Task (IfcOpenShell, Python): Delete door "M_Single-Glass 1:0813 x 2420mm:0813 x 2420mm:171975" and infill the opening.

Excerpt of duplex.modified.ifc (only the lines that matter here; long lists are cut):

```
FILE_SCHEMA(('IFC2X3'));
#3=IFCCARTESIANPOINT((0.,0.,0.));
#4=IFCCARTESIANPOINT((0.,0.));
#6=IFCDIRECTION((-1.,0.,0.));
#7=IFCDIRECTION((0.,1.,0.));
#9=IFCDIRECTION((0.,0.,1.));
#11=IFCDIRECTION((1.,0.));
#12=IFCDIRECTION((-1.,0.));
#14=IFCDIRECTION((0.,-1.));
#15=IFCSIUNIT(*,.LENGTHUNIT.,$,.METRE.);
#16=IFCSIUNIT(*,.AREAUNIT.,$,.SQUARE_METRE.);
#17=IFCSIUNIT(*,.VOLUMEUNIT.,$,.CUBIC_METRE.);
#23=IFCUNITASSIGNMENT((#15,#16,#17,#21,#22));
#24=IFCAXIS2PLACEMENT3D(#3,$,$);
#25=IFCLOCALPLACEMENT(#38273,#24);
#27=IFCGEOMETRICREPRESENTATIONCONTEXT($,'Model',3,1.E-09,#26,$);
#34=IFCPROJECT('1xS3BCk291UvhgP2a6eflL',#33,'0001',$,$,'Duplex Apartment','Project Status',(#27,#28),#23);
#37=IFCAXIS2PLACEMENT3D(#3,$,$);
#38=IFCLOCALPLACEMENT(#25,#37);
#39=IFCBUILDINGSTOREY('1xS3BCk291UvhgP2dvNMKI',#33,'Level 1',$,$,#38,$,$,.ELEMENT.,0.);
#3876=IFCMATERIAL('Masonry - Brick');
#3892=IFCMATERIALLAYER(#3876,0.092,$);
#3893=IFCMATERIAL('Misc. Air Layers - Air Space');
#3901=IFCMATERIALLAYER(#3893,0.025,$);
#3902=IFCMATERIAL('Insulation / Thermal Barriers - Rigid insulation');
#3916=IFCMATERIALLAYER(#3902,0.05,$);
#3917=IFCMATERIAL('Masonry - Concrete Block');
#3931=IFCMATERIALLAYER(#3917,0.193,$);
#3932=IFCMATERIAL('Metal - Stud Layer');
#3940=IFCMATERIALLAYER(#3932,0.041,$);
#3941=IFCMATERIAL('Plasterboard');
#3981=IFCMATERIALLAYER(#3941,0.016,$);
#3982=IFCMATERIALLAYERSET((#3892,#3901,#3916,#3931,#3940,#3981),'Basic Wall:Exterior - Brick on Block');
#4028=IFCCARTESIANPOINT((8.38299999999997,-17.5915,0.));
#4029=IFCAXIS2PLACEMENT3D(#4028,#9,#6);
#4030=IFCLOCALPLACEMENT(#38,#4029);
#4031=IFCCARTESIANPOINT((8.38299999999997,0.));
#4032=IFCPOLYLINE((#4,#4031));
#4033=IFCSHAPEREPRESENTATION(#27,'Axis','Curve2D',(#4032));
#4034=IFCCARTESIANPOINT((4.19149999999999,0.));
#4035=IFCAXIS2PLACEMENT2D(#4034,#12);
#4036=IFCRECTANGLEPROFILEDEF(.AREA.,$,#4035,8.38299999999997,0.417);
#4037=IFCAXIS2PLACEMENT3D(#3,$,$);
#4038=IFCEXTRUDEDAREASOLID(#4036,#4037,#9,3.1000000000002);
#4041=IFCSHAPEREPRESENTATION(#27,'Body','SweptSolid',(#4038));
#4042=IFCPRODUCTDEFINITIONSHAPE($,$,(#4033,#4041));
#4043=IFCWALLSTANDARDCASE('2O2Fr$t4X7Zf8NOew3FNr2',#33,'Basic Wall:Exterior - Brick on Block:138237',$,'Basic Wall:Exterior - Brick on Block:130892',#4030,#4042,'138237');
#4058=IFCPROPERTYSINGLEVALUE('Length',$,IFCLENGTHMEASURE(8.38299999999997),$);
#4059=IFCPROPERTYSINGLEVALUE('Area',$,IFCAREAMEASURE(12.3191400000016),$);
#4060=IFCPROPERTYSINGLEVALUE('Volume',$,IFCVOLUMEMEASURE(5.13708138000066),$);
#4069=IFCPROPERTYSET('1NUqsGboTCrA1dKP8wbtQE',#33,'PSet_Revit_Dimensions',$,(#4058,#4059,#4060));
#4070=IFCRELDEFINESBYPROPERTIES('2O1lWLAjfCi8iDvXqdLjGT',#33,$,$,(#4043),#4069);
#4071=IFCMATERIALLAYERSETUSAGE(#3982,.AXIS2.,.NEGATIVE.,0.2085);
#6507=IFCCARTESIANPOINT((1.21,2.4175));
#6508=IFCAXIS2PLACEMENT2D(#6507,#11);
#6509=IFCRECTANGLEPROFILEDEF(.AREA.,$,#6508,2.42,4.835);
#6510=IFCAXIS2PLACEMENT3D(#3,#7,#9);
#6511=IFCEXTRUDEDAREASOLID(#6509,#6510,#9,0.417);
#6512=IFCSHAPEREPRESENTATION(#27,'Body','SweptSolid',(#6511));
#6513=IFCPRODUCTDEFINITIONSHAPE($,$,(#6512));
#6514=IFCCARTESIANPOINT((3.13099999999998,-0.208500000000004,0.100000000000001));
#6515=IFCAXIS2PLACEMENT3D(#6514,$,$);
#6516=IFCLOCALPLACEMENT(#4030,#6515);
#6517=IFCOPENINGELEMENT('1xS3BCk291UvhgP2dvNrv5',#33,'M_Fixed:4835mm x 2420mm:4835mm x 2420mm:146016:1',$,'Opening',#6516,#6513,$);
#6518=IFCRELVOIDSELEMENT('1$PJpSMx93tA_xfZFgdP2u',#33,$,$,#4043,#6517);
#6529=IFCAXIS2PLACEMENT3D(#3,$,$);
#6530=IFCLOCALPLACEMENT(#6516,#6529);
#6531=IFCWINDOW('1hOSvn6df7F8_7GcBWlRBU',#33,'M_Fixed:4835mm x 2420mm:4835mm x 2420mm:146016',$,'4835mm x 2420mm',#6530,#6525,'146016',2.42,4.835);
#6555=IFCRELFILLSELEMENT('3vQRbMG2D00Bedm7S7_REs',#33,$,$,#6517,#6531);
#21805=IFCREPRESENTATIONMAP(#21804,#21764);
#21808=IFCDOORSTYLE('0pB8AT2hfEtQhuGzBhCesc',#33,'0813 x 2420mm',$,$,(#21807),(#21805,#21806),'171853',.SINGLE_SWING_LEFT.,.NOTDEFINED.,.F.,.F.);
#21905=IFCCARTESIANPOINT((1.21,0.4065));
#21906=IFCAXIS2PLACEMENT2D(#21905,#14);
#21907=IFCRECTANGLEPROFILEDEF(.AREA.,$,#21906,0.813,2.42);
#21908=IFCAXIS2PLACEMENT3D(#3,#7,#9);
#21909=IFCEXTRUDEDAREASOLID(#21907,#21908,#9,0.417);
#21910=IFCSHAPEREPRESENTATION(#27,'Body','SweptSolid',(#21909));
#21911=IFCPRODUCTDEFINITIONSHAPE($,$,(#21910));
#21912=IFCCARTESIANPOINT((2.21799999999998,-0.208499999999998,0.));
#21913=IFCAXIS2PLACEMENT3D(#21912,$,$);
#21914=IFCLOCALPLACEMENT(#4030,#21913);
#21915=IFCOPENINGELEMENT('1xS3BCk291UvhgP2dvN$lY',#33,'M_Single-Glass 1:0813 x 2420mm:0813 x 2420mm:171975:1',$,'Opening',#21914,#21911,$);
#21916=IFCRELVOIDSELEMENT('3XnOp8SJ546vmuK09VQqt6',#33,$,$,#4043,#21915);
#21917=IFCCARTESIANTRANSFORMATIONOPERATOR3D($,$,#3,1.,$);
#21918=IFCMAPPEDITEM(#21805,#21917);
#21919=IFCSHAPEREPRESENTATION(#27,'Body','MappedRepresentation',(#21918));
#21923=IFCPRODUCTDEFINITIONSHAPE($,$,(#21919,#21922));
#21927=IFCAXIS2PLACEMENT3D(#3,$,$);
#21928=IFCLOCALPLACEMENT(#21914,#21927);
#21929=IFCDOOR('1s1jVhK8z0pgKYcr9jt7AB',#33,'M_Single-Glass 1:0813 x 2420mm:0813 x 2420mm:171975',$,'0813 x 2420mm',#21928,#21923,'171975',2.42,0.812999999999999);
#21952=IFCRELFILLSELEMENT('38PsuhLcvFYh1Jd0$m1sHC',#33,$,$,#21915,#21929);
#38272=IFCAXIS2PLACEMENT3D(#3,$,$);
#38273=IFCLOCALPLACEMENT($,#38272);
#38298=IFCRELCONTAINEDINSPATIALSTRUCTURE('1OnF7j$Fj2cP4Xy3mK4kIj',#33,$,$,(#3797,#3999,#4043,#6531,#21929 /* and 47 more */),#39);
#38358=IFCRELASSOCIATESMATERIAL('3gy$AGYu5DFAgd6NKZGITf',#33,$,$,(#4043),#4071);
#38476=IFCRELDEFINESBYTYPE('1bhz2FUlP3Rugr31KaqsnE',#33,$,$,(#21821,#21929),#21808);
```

```python
import ifcopenshell
import ifcopenshell.api.feature
import ifcopenshell.api.pset
import ifcopenshell.api.root
import ifcopenshell.geom
import ifcopenshell.util.element
import ifcopenshell.util.shape
import ifcopenshell.util.unit

model = ifcopenshell.open("duplex.modified.ifc")
area_scale = ifcopenshell.util.unit.calculate_unit_scale(model, "AREAUNIT")
volume_scale = ifcopenshell.util.unit.calculate_unit_scale(model, "VOLUMEUNIT")
settings = ifcopenshell.geom.settings()


def volume(element):
    """Net volume in cubic metres, openings subtracted."""
    shape = ifcopenshell.geom.create_shape(settings, element)
    return ifcopenshell.util.shape.get_volume(shape.geometry)


door = model.by_id(21929)
opening = door.FillsVoids[0].RelatingOpeningElement
wall = opening.VoidsElements[0].RelatingBuildingElement
before = volume(wall)

ifcopenshell.api.root.remove_product(model, product=door)
ifcopenshell.api.feature.remove_feature(model, feature=opening)

after = volume(wall)
thickness = 0.417  # wall thickness in metres

# Update the wall's stored quantities.
pset = model.by_id(ifcopenshell.util.element.get_pset(wall, "PSet_Revit_Dimensions", should_inherit=False)["id"])
ifcopenshell.api.pset.edit_pset(model, pset=pset, properties={
    "Area": model.create_entity("IfcAreaMeasure", after / thickness / area_scale),
    "Volume": model.create_entity("IfcVolumeMeasure", after / volume_scale),
})

print(f"wall volume {before:.3f} -> {after:.3f} m3")

model.write("duplex.modified_updated.ifc")
```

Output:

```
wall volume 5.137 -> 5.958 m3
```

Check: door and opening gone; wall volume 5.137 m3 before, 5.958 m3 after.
